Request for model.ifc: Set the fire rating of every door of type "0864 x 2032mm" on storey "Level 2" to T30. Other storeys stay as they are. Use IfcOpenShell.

First a look at what the model holds.

```python
import ifcopenshell
import ifcopenshell.util.element

model = ifcopenshell.open("model.ifc")
print(model.schema)
storey = next(s for s in model.by_type("IfcBuildingStorey") if s.Name == "Level 2")
doors = [e for e in ifcopenshell.util.element.get_decomposition(storey) if e.is_a("IfcDoor")]
seen = {}
for e in doors:
    element_type = ifcopenshell.util.element.get_type(e)
    key = (element_type.Name if element_type != e and element_type else None, ifcopenshell.util.element.get_pset(e, "Pset_DoorCommon", "FireRating"))
    seen[key] = seen.get(key, 0) + 1
for (name, value), count in sorted(seen.items(), key=str):
    print(count, "x", name, "|", value)
```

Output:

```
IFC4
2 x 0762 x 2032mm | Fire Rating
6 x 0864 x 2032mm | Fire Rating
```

```python
import ifcopenshell
import ifcopenshell.api.pset
import ifcopenshell.util.element

model = ifcopenshell.open("model.ifc")

storey = next(s for s in model.by_type("IfcBuildingStorey") if s.Name == "Level 2")
doors = [e for e in ifcopenshell.util.element.get_decomposition(storey) if e.is_a("IfcDoor")]

count = 0
for e in doors:
    element_type = ifcopenshell.util.element.get_type(e)
    if element_type in (None, e) or element_type.Name != "0864 x 2032mm":
        continue
    # add_pset returns the element's existing set when there is one.
    pset = ifcopenshell.api.pset.add_pset(model, product=e, name="Pset_DoorCommon")
    ifcopenshell.api.pset.edit_pset(model, pset=pset, properties={"FireRating": "T30"})
    count += 1

print(count, "doors updated")

model.write("model_edited.ifc")
```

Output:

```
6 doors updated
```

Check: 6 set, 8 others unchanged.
